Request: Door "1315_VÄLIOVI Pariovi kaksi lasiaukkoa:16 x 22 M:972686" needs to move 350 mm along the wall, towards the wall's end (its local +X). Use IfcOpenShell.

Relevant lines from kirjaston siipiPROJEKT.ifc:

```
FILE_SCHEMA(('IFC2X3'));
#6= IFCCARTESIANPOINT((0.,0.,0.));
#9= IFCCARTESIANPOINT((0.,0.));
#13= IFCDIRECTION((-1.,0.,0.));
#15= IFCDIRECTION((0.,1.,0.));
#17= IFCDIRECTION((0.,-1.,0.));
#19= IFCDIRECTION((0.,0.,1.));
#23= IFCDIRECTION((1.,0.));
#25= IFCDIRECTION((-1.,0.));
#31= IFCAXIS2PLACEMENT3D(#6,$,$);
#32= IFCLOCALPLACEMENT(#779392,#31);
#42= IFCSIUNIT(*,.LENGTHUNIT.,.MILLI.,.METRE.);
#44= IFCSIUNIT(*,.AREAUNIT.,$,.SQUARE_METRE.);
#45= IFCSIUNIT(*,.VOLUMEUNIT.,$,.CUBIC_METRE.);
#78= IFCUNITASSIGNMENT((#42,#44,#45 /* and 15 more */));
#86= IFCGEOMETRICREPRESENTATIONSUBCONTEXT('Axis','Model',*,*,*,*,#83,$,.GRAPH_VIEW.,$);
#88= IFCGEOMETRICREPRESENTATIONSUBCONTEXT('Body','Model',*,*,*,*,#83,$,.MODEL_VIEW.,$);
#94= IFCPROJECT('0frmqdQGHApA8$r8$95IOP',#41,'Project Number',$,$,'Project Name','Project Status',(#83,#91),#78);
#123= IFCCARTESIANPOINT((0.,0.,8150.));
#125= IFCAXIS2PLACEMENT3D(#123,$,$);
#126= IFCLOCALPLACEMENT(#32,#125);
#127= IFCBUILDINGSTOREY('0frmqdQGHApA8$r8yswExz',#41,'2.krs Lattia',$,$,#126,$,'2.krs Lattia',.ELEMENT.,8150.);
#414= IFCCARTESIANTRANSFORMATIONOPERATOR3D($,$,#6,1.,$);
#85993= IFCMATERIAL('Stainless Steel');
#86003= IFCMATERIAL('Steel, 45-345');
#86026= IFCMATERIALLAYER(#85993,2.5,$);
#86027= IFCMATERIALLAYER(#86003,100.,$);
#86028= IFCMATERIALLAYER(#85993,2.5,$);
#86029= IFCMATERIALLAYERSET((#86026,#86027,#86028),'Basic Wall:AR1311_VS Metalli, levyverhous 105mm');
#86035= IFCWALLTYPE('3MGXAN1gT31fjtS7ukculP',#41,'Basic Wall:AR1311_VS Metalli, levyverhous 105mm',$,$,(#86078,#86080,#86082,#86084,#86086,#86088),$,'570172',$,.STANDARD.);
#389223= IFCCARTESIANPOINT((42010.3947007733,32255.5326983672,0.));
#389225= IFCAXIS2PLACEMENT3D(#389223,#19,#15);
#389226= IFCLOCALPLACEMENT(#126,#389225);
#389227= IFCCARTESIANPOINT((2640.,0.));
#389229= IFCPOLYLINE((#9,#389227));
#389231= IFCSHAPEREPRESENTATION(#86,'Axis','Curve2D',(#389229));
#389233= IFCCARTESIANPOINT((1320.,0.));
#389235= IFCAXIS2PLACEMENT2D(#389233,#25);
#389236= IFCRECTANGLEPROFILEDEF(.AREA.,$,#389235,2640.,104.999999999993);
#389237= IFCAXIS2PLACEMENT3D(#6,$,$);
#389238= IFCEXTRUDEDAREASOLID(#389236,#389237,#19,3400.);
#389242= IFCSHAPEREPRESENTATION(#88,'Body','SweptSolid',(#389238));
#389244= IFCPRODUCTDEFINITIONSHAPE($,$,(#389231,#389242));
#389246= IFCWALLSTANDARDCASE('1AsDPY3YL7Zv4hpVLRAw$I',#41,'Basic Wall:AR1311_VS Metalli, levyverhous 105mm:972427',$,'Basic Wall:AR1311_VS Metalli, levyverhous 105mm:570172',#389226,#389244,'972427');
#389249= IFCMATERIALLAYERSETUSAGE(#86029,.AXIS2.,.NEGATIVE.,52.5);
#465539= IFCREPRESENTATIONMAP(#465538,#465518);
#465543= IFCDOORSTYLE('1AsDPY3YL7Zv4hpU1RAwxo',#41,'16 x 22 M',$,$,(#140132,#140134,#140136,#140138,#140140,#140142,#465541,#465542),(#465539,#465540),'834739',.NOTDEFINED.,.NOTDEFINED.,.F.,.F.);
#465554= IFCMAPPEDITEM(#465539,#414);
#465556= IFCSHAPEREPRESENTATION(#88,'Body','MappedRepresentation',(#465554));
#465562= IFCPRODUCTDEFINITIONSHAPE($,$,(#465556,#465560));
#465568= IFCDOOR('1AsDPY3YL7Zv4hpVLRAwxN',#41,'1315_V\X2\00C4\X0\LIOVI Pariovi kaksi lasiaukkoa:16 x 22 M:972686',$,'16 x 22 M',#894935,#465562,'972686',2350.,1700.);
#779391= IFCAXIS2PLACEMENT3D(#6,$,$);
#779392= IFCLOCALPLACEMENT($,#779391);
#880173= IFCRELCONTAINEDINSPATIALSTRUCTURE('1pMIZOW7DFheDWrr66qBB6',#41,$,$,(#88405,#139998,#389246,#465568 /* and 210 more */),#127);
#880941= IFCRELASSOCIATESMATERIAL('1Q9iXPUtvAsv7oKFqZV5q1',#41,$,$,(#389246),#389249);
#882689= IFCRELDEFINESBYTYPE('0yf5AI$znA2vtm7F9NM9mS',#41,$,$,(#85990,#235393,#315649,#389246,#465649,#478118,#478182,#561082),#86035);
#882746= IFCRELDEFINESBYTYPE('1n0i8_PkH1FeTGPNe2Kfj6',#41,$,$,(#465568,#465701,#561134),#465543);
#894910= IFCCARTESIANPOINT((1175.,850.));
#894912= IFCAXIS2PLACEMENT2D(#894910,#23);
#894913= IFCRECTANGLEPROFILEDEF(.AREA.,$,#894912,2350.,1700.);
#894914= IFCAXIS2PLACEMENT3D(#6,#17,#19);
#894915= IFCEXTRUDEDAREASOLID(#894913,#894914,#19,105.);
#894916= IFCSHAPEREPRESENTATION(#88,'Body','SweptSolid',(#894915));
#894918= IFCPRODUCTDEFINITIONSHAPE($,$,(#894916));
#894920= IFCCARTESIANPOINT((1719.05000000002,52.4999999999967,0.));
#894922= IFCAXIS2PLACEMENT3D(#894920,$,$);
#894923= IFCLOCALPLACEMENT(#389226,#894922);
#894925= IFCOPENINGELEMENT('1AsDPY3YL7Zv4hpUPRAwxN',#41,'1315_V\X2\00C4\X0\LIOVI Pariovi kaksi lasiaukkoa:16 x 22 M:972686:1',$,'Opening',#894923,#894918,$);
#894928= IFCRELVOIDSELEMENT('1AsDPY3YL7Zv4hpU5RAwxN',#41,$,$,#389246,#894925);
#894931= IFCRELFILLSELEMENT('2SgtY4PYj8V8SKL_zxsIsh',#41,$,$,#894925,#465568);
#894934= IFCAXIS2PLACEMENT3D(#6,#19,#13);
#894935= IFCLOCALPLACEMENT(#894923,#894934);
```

```python
import ifcopenshell
import ifcopenshell.api.geometry
import ifcopenshell.util.placement

model = ifcopenshell.open("kirjaston siipiPROJEKT.ifc")

door = model.by_id(465568)
opening = door.FillsVoids[0].RelatingOpeningElement
wall = opening.VoidsElements[0].RelatingBuildingElement

wall_matrix = ifcopenshell.util.placement.get_local_placement(wall.ObjectPlacement)
shift = wall_matrix[:3, 0] * 350.0
before = ifcopenshell.util.placement.get_local_placement(door.ObjectPlacement)[:3, 3].copy()

# The door is placed relative to its opening, so it follows when the opening moves.
matrix = ifcopenshell.util.placement.get_local_placement(opening.ObjectPlacement)
matrix[:3, 3] += shift
ifcopenshell.api.geometry.edit_object_placement(
    model, product=opening, matrix=matrix, is_si=False, should_transform_children=True
)

after = ifcopenshell.util.placement.get_local_placement(door.ObjectPlacement)[:3, 3]
print("door moved by", (after - before).round(3) + 0.0)

model.write("kirjaston siipiPROJEKT_v2.ifc")
```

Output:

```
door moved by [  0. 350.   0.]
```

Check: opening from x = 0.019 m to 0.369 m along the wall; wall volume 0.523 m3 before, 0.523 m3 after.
